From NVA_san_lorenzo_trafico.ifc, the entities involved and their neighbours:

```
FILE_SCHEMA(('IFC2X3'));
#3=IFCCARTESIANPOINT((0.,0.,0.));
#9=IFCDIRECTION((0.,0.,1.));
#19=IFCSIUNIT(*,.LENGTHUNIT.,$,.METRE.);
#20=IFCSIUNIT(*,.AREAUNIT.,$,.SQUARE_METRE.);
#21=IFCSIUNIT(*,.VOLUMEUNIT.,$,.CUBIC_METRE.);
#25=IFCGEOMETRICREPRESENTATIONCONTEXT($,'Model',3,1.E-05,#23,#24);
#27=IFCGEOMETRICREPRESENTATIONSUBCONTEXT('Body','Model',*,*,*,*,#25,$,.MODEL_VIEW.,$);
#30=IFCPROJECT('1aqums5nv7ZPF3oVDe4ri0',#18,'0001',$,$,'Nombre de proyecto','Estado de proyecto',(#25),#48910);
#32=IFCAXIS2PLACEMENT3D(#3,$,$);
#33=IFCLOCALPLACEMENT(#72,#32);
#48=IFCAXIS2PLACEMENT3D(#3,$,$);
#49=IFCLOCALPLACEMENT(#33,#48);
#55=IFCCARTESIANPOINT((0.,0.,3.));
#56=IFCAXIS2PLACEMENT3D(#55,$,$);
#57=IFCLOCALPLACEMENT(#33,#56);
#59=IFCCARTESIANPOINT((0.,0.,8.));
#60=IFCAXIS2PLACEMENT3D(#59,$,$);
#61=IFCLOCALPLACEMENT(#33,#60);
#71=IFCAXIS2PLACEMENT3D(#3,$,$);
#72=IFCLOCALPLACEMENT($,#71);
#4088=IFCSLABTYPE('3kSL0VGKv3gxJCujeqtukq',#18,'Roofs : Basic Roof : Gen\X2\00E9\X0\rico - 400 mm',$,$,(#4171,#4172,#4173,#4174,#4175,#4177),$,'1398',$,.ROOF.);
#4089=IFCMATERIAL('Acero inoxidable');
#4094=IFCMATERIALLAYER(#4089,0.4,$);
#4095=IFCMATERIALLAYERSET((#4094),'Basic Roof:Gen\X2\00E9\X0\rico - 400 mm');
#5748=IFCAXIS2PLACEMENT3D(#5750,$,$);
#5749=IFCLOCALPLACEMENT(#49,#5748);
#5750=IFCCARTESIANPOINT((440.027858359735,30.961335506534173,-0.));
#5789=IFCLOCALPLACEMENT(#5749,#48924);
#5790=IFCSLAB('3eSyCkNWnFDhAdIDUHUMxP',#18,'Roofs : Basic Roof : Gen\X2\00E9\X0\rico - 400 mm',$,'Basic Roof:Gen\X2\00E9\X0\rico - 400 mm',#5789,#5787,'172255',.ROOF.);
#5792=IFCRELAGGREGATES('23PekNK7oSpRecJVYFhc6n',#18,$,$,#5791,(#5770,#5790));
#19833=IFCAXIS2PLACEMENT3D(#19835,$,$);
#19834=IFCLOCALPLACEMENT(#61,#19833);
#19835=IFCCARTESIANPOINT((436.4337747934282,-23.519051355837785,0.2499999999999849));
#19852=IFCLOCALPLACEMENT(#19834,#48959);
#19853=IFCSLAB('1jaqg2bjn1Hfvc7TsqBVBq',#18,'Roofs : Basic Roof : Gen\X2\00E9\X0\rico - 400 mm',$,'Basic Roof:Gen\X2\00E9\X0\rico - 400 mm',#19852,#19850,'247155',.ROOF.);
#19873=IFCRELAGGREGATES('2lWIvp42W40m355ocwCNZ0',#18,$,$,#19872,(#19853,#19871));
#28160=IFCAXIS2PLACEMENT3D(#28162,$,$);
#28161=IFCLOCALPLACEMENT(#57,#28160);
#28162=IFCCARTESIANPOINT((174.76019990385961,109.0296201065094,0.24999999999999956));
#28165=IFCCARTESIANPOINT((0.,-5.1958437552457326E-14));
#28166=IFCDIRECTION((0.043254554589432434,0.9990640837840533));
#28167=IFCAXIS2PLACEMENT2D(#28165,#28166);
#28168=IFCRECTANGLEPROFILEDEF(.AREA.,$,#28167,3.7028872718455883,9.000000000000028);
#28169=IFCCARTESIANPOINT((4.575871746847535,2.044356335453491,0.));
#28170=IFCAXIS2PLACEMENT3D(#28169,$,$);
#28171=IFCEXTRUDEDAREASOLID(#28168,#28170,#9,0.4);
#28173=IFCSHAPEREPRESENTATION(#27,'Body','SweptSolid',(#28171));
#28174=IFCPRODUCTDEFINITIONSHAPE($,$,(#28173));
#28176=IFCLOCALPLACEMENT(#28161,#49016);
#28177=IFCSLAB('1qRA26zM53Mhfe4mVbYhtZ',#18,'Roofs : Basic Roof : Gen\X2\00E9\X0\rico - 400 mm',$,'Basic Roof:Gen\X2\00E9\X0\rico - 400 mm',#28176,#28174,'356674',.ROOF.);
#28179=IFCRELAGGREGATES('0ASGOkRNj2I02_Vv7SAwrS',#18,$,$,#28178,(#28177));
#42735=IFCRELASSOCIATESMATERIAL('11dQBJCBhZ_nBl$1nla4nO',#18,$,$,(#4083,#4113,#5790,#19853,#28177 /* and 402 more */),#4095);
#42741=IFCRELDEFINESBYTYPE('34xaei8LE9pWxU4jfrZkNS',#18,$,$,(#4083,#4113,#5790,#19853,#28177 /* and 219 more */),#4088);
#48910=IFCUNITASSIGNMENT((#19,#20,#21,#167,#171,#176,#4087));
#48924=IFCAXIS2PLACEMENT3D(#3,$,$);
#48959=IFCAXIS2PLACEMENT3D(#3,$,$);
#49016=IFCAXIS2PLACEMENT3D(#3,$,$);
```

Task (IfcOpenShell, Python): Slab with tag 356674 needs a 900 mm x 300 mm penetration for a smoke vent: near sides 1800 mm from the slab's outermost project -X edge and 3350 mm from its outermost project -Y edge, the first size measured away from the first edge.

```python
import numpy as np
import ifcopenshell
import ifcopenshell.api.feature
import ifcopenshell.api.geometry
import ifcopenshell.api.root
import ifcopenshell.geom
import ifcopenshell.util.placement
import ifcopenshell.util.representation
import ifcopenshell.util.shape
import ifcopenshell.util.unit

model = ifcopenshell.open("NVA_san_lorenzo_trafico.ifc")
unit_scale = ifcopenshell.util.unit.calculate_unit_scale(model)
settings = ifcopenshell.geom.settings()


def volume(element):
    """Net volume in cubic metres, openings subtracted."""
    shape = ifcopenshell.geom.create_shape(settings, element)
    return ifcopenshell.util.shape.get_volume(shape.geometry)


slab = model.by_id(28177)
before = volume(slab)

# Extent in the slab's own axes, in metres. The edges named are its -X and -Y sides.
slab_shape = ifcopenshell.geom.create_shape(settings, slab)
vertices = ifcopenshell.util.shape.get_vertices(slab_shape.geometry)
x_min, y_min, bottom = vertices.min(axis=0)
top = vertices[:, 2].max()

opening = ifcopenshell.api.root.create_entity(model, ifc_class="IfcOpeningElement", name="Smoke vent opening")
context = ifcopenshell.util.representation.get_context(model, "Model", "Body", "MODEL_VIEW")
width, depth = 0.9, 0.3
outline = [(0.0, 0.0), (width, 0.0), (width, depth), (0.0, depth), (0.0, 0.0)]
# Overshoot both faces by 50 mm so the cut is clean.
shape = ifcopenshell.api.geometry.add_slab_representation(
    model, context=context, depth=top - bottom + 0.1, polyline=outline
)
ifcopenshell.api.geometry.assign_representation(model, product=opening, representation=shape)

matrix = ifcopenshell.util.placement.get_local_placement(slab.ObjectPlacement)
matrix[:, 3] = matrix @ np.append(np.array([x_min + 1.8, y_min + 3.35, bottom - 0.05]) / unit_scale, 1.0)
ifcopenshell.api.geometry.edit_object_placement(model, product=opening, matrix=matrix, is_si=False)
ifcopenshell.api.feature.add_feature(model, feature=opening, element=slab)

after = volume(slab)

print(f"slab volume {before:.3f} -> {after:.3f} m3")

model.write("NVA_san_lorenzo_trafico-out.ifc")
```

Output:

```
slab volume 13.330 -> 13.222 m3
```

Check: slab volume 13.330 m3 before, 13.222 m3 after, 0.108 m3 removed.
